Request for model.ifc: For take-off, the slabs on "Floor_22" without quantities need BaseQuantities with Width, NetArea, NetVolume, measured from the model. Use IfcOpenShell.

First a look at what the model holds.

```python
import ifcopenshell
import ifcopenshell.util.element
import ifcopenshell.util.unit

model = ifcopenshell.open("model.ifc")
print(model.schema)
for unit_type in ("LENGTHUNIT", "AREAUNIT", "VOLUMEUNIT"):
    print(unit_type, ifcopenshell.util.unit.calculate_unit_scale(model, unit_type))
storey = next(s for s in model.by_type("IfcBuildingStorey") if s.Name == "Floor_22")
slabs = [e for e in ifcopenshell.util.element.get_decomposition(storey) if e.is_a("IfcSlab")]
for e in sorted(slabs, key=lambda e: e.id()):
    print(e.id(), e.is_a(), e.Name, list(ifcopenshell.util.element.get_psets(e, qtos_only=True)), sep=" | ")
```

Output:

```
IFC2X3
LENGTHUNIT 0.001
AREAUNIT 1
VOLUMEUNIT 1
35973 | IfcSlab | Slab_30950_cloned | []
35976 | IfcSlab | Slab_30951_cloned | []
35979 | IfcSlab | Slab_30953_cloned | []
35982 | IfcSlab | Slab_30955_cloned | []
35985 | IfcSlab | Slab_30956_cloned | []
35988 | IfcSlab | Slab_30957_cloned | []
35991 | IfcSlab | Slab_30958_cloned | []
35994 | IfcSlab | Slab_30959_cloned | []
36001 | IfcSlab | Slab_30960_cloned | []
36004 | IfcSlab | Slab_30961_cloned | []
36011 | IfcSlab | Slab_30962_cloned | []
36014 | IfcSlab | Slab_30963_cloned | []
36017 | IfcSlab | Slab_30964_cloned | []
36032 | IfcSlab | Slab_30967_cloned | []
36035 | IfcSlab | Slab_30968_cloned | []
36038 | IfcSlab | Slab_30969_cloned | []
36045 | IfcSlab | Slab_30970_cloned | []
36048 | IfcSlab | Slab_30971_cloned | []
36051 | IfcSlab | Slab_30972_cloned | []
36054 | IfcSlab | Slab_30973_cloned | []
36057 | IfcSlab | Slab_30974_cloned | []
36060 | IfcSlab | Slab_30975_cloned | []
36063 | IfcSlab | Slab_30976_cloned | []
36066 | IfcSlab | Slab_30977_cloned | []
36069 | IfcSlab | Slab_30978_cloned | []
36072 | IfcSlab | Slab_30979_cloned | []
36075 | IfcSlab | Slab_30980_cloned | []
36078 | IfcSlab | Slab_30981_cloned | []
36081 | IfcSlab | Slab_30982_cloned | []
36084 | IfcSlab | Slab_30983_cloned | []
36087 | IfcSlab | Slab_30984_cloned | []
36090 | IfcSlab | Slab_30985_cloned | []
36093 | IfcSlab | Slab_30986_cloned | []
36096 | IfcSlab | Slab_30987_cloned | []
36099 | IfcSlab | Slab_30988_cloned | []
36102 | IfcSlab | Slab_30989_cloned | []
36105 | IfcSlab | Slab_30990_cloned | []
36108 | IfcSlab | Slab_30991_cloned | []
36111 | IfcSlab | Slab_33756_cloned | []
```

```python
import ifcopenshell
import ifcopenshell.api.pset
import ifcopenshell.geom
import ifcopenshell.util.element
import ifcopenshell.util.shape
import ifcopenshell.util.unit

model = ifcopenshell.open("model.ifc")
unit_scale = ifcopenshell.util.unit.calculate_unit_scale(model)
area_scale = ifcopenshell.util.unit.calculate_unit_scale(model, "AREAUNIT")
volume_scale = ifcopenshell.util.unit.calculate_unit_scale(model, "VOLUMEUNIT")
settings = ifcopenshell.geom.settings()

storey = next(s for s in model.by_type("IfcBuildingStorey") if s.Name == "Floor_22")
slabs = [e for e in ifcopenshell.util.element.get_decomposition(storey) if e.is_a("IfcSlab")]

for e in sorted(slabs, key=lambda e: e.id()):
    if ifcopenshell.util.element.get_psets(e, qtos_only=True, should_inherit=False):
        continue
    # Geometry comes back in metres, in the element's own axes.
    shape = ifcopenshell.geom.create_shape(settings, e)
    values = {
        "Width": ifcopenshell.util.shape.get_z(shape.geometry) / unit_scale,
        "NetArea": ifcopenshell.util.shape.get_footprint_area(shape.geometry) / area_scale,
        "NetVolume": ifcopenshell.util.shape.get_volume(shape.geometry) / volume_scale,
    }
    qto = ifcopenshell.api.pset.add_qto(model, product=e, name="BaseQuantities")
    ifcopenshell.api.pset.edit_qto(model, qto=qto, properties=values)
    print(e.id(), {k: round(v, 3) for k, v in values.items()})

model.write("model_rev.ifc")
```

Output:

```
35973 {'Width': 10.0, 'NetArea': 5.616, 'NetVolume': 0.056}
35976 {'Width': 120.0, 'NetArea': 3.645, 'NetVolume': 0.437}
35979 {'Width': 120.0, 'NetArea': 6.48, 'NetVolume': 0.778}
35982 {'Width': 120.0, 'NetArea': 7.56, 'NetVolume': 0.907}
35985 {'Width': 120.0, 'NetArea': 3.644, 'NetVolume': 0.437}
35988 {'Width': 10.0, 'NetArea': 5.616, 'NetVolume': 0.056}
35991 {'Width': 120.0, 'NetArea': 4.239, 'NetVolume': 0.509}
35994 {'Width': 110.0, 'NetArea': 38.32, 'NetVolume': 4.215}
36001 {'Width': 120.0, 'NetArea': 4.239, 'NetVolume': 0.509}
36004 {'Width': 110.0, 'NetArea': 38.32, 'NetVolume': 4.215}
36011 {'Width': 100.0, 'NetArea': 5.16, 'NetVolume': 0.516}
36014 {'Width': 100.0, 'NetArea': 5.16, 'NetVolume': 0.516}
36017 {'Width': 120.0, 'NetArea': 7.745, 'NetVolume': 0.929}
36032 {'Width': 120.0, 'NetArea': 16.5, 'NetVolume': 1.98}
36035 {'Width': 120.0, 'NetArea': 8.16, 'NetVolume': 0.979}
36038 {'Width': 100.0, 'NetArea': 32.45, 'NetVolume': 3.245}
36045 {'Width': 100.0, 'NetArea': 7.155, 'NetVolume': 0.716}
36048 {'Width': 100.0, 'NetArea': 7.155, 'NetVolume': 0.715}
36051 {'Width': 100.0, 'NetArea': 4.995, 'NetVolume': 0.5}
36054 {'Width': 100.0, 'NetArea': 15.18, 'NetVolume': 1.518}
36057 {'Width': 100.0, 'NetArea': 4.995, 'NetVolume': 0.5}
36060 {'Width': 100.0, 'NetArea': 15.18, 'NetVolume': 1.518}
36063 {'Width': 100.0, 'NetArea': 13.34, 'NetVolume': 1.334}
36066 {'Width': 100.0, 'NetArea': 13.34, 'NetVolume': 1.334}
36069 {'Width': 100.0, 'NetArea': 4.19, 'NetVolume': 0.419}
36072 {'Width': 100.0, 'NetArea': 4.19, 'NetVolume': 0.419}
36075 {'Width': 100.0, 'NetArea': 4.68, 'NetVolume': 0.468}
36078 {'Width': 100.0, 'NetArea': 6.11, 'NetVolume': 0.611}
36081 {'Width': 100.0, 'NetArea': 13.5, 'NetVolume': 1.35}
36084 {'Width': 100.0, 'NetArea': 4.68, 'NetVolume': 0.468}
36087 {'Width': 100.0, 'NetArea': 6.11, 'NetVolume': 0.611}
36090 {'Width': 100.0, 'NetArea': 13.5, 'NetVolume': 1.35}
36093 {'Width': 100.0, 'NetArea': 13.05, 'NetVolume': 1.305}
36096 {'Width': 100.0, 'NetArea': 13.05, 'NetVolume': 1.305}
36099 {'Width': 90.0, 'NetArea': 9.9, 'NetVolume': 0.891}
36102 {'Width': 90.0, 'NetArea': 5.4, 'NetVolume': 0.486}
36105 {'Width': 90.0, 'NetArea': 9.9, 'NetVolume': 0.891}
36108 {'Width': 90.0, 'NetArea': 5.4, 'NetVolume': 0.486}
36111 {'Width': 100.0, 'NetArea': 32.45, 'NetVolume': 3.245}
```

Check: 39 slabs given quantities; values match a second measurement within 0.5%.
